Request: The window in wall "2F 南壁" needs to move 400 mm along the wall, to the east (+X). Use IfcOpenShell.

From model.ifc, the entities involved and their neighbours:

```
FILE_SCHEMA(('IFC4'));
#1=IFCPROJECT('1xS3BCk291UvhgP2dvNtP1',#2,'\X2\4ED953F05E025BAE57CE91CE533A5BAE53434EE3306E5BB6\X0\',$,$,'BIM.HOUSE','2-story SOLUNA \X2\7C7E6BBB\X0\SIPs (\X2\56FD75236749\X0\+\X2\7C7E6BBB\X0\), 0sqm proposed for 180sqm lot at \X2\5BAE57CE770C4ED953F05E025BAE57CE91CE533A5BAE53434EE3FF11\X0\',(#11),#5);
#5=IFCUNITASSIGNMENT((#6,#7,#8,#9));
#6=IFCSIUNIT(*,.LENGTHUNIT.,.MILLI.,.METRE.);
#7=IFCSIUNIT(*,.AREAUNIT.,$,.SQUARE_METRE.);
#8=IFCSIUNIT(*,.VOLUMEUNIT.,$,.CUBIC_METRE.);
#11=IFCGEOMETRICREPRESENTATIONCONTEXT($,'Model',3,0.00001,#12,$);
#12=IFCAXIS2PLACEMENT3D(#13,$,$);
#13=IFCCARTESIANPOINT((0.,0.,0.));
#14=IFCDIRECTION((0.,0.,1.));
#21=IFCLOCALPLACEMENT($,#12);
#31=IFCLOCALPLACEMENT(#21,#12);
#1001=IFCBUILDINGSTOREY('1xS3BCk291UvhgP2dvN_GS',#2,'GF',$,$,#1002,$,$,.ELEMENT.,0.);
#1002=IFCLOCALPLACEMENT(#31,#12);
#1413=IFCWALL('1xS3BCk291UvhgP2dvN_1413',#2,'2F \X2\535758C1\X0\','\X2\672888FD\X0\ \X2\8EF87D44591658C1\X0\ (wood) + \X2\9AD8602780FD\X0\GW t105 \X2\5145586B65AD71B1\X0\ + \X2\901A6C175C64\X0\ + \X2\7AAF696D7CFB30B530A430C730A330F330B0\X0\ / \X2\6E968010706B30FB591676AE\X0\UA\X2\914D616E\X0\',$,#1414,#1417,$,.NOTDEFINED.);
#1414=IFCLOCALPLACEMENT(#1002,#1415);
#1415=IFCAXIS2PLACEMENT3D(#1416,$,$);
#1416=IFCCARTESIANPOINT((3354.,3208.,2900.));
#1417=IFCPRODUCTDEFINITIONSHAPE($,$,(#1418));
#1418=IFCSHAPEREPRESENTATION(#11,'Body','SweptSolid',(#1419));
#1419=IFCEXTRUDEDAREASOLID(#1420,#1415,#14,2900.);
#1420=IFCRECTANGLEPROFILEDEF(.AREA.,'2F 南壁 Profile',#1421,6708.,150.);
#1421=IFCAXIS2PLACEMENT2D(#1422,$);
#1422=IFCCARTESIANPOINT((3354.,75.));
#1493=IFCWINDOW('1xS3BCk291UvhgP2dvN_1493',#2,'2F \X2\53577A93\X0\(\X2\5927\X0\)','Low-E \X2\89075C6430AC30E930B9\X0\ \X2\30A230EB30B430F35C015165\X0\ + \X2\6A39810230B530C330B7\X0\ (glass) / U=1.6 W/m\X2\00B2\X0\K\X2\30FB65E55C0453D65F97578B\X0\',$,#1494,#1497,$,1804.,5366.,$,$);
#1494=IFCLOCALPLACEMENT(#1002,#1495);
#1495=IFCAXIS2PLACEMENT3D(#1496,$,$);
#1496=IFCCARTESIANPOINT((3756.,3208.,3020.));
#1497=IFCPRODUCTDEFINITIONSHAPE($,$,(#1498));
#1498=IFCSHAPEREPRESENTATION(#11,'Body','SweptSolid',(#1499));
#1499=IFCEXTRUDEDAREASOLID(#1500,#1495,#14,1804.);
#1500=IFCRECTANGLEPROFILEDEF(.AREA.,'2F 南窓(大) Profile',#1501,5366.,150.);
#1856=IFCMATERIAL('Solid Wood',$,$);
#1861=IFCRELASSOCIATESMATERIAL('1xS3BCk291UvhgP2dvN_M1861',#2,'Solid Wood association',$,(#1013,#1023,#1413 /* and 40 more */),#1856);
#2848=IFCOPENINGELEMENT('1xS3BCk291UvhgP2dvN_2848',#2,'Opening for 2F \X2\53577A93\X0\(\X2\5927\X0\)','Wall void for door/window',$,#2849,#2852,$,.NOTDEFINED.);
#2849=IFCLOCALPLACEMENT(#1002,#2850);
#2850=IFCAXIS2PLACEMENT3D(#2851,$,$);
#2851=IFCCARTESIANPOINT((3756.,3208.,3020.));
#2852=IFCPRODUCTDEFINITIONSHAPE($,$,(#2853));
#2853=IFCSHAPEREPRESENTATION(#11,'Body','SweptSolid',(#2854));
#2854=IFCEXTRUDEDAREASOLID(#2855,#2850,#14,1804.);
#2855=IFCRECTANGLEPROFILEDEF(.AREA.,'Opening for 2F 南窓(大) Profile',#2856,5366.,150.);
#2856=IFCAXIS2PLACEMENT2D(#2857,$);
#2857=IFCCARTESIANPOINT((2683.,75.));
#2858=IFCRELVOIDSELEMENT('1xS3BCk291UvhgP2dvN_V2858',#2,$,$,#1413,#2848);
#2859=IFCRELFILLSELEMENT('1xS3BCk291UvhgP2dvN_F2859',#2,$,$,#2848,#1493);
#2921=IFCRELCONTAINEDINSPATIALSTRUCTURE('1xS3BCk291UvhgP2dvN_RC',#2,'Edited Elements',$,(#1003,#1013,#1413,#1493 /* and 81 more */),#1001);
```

```python
import ifcopenshell
import ifcopenshell.api.geometry
import ifcopenshell.util.placement

model = ifcopenshell.open("model.ifc")

window = model.by_id(1493)
opening = window.FillsVoids[0].RelatingOpeningElement
wall = opening.VoidsElements[0].RelatingBuildingElement

wall_matrix = ifcopenshell.util.placement.get_local_placement(wall.ObjectPlacement)
shift = wall_matrix[:3, 0] * 400.0
before = ifcopenshell.util.placement.get_local_placement(window.ObjectPlacement)[:3, 3].copy()

# The window is not placed relative to its opening, so move both.
for product in (opening, window):
    matrix = ifcopenshell.util.placement.get_local_placement(product.ObjectPlacement)
    matrix[:3, 3] += shift
    ifcopenshell.api.geometry.edit_object_placement(model, product=product, matrix=matrix, is_si=False)

after = ifcopenshell.util.placement.get_local_placement(window.ObjectPlacement)[:3, 3]
print("window moved by", (after - before).round(3) + 0.0)

model.write("model_rev.ifc")
```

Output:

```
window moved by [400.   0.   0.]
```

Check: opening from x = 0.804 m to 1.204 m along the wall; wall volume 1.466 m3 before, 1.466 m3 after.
